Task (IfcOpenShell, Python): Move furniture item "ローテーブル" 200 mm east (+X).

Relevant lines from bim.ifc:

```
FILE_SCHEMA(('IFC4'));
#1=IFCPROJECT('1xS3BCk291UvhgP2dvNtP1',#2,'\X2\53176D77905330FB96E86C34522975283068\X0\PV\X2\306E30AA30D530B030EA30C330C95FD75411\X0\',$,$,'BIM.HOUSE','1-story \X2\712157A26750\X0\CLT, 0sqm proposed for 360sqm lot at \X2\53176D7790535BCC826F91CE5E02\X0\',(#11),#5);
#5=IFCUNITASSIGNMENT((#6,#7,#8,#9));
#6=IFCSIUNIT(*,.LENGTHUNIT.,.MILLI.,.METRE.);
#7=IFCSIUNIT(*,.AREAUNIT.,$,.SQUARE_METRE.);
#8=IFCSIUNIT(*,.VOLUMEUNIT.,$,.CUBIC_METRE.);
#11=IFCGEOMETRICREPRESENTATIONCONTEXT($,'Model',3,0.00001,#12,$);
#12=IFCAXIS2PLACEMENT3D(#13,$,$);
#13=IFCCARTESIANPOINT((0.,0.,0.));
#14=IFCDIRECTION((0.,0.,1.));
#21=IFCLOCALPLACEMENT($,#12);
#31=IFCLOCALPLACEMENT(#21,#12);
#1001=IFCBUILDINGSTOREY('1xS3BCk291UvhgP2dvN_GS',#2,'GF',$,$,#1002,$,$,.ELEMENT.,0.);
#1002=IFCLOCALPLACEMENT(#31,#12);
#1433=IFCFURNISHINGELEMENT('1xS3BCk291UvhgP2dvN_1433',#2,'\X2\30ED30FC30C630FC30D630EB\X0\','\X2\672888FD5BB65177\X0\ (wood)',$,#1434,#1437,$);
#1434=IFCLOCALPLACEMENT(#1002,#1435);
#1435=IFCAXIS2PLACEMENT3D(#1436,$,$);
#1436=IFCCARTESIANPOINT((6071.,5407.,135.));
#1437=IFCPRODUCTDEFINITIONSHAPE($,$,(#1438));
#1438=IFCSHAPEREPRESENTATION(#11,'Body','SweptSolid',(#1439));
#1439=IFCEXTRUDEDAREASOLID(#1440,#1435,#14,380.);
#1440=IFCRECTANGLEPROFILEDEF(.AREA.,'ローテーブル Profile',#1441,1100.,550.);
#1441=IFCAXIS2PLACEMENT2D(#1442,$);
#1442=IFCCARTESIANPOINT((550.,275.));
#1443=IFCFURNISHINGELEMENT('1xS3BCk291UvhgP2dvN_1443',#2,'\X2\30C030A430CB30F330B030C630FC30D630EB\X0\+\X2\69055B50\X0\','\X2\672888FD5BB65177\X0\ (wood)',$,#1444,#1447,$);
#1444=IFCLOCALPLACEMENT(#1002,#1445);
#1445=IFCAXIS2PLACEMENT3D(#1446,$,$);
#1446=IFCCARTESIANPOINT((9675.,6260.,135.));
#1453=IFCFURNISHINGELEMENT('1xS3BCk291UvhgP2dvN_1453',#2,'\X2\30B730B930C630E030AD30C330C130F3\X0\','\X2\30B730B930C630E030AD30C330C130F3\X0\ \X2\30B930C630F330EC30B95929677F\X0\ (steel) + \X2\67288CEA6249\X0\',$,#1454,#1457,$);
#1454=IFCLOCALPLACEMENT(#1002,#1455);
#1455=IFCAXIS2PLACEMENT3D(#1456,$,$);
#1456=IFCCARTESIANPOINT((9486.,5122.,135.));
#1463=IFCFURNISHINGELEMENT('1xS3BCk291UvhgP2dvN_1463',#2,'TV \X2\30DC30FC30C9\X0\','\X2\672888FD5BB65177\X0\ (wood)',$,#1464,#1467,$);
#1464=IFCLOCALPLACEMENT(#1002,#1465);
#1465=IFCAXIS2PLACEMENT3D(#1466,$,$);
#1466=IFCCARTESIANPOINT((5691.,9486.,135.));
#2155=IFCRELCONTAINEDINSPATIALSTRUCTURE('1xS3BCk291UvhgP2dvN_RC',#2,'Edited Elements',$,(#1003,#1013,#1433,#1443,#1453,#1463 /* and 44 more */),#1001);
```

```python
import ifcopenshell
import ifcopenshell.api.geometry
import ifcopenshell.util.placement
import ifcopenshell.util.unit

model = ifcopenshell.open("bim.ifc")
unit_scale = ifcopenshell.util.unit.calculate_unit_scale(model)

item = model.by_guid("1xS3BCk291UvhgP2dvN_1433")
matrix = ifcopenshell.util.placement.get_local_placement(item.ObjectPlacement)
matrix[0, 3] += 0.2 / unit_scale
ifcopenshell.api.geometry.edit_object_placement(model, product=item, matrix=matrix, is_si=False)

print(ifcopenshell.util.placement.get_local_placement(item.ObjectPlacement).round(3) + 0.0)

model.write("bim_updated.ifc")
```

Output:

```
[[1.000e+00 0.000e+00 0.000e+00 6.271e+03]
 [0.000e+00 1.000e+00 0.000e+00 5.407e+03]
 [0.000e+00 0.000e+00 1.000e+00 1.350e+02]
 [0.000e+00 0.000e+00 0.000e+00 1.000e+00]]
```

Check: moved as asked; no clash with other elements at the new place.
